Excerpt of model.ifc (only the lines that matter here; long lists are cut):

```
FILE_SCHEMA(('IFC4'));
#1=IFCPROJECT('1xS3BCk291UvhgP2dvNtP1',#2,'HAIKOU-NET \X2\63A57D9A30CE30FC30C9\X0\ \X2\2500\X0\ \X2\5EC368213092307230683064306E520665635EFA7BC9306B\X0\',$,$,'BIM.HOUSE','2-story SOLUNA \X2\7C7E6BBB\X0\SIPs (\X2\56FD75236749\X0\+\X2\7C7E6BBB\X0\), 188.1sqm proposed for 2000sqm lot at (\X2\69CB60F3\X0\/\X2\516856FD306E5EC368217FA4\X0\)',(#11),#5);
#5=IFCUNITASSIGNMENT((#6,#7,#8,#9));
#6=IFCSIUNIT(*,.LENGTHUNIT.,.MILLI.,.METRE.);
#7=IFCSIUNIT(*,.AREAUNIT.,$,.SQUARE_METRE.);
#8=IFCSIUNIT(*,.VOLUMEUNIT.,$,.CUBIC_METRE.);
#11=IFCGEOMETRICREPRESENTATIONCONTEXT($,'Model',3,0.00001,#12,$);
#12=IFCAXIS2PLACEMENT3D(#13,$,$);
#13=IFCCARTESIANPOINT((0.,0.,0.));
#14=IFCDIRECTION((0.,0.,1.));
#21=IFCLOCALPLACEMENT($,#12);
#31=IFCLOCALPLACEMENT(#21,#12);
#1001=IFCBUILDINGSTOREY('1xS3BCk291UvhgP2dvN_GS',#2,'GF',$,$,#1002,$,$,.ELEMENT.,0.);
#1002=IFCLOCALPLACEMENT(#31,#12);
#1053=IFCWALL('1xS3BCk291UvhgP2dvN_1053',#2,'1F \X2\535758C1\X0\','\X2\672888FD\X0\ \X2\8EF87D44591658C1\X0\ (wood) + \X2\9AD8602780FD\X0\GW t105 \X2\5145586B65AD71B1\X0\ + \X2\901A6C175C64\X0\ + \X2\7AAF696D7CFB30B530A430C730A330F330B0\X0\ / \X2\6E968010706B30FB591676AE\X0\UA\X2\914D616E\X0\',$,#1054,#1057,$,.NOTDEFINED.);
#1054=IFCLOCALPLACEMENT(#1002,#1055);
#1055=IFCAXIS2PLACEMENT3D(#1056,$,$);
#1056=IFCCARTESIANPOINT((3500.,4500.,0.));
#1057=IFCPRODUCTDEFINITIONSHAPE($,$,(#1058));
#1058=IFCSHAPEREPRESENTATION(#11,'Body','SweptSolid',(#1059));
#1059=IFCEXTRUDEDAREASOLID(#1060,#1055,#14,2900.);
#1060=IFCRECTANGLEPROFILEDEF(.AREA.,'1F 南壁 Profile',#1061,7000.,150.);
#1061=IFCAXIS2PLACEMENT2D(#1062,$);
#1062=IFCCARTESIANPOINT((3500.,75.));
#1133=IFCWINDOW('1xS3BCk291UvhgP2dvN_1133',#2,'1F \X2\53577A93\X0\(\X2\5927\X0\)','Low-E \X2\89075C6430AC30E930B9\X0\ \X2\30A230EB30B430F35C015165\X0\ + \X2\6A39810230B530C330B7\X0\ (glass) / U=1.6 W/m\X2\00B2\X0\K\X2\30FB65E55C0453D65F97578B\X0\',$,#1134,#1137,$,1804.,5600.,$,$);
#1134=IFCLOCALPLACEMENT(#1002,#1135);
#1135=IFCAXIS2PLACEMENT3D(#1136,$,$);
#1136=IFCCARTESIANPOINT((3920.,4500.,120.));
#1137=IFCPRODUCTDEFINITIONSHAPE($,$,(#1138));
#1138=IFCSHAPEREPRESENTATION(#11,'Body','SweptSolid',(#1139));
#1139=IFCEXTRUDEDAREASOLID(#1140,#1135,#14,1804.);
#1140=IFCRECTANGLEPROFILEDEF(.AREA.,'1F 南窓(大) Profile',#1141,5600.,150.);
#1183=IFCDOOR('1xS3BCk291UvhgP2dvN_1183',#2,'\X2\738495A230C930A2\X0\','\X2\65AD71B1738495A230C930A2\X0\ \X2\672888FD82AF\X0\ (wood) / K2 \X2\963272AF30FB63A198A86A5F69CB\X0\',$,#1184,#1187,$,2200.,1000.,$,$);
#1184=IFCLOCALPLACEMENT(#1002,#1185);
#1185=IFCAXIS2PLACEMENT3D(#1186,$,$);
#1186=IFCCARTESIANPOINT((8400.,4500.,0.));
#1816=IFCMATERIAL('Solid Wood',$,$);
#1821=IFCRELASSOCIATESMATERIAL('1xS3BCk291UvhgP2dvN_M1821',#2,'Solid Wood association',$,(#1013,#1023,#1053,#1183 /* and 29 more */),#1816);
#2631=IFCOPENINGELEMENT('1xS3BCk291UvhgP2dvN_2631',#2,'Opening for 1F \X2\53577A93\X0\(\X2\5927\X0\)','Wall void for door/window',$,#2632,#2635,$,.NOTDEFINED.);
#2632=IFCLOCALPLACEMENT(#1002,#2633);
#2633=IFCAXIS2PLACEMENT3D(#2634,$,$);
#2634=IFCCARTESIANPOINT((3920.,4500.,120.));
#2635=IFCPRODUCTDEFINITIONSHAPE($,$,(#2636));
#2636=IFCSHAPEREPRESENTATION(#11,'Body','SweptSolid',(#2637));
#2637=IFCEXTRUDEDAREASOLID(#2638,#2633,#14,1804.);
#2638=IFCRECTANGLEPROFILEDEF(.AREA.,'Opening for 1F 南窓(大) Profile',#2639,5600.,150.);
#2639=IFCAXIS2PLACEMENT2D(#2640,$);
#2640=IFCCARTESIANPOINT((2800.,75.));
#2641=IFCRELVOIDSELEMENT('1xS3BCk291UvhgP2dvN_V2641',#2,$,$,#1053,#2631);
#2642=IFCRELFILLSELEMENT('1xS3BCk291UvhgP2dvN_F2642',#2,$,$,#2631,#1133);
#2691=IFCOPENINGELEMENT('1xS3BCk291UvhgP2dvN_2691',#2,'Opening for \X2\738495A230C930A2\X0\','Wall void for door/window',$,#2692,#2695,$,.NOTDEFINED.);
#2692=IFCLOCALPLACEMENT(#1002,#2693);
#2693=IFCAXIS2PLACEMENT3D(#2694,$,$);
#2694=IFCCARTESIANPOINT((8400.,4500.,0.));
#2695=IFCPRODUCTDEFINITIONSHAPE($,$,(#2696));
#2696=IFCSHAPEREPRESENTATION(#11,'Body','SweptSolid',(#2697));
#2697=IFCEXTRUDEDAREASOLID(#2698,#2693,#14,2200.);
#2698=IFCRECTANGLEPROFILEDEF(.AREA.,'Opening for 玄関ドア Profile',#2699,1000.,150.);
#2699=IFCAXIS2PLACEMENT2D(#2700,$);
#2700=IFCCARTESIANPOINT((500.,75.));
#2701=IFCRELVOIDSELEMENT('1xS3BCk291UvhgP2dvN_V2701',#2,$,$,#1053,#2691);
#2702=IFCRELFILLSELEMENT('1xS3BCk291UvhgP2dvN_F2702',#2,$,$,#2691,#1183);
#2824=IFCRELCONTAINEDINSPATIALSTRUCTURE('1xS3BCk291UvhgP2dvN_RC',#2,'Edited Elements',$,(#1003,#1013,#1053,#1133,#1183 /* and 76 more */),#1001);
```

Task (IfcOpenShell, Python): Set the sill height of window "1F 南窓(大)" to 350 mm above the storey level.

```python
import numpy as np
import ifcopenshell
import ifcopenshell.api.geometry
import ifcopenshell.geom
import ifcopenshell.util.element
import ifcopenshell.util.placement
import ifcopenshell.util.shape
import ifcopenshell.util.unit

model = ifcopenshell.open("model.ifc")
unit_scale = ifcopenshell.util.unit.calculate_unit_scale(model)

window = model.by_guid("1xS3BCk291UvhgP2dvN_1133")
opening = window.FillsVoids[0].RelatingOpeningElement
storey = ifcopenshell.util.element.get_container(window, ifc_class="IfcBuildingStorey")
level = ifcopenshell.util.placement.get_local_placement(storey.ObjectPlacement)[2, 3]

# The opening's origin need not be at the sill, so measure its lowest point.
shape = ifcopenshell.geom.create_shape(ifcopenshell.geom.settings(), opening)
bottom = ifcopenshell.util.shape.get_shape_bottom_elevation(shape, shape.geometry) / unit_scale
dz = level + 350.0 - bottom

shift = np.array([0.0, 0.0, dz])
# The window is not placed relative to its opening, so move both.
for product in (opening, window):
    matrix = ifcopenshell.util.placement.get_local_placement(product.ObjectPlacement)
    matrix[:3, 3] += shift
    ifcopenshell.api.geometry.edit_object_placement(model, product=product, matrix=matrix, is_si=False)

print(f"moved by {dz * unit_scale:+.3f} m")

model.write("model-out.ifc")
```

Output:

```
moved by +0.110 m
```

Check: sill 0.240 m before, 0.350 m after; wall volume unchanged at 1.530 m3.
